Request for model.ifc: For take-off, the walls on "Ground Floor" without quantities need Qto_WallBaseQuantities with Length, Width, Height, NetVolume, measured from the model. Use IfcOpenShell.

First a look at what the model holds.

```python
import ifcopenshell
import ifcopenshell.util.element
import ifcopenshell.util.unit

model = ifcopenshell.open("model.ifc")
print(model.schema)
for unit_type in ("LENGTHUNIT", "AREAUNIT", "VOLUMEUNIT"):
    print(unit_type, ifcopenshell.util.unit.calculate_unit_scale(model, unit_type))
storey = next(s for s in model.by_type("IfcBuildingStorey") if s.Name == "Ground Floor")
walls = [e for e in ifcopenshell.util.element.get_decomposition(storey) if e.is_a("IfcWall")]
for e in sorted(walls, key=lambda e: e.id()):
    print(e.id(), e.is_a(), e.Name, list(ifcopenshell.util.element.get_psets(e, qtos_only=True)), sep=" | ")
```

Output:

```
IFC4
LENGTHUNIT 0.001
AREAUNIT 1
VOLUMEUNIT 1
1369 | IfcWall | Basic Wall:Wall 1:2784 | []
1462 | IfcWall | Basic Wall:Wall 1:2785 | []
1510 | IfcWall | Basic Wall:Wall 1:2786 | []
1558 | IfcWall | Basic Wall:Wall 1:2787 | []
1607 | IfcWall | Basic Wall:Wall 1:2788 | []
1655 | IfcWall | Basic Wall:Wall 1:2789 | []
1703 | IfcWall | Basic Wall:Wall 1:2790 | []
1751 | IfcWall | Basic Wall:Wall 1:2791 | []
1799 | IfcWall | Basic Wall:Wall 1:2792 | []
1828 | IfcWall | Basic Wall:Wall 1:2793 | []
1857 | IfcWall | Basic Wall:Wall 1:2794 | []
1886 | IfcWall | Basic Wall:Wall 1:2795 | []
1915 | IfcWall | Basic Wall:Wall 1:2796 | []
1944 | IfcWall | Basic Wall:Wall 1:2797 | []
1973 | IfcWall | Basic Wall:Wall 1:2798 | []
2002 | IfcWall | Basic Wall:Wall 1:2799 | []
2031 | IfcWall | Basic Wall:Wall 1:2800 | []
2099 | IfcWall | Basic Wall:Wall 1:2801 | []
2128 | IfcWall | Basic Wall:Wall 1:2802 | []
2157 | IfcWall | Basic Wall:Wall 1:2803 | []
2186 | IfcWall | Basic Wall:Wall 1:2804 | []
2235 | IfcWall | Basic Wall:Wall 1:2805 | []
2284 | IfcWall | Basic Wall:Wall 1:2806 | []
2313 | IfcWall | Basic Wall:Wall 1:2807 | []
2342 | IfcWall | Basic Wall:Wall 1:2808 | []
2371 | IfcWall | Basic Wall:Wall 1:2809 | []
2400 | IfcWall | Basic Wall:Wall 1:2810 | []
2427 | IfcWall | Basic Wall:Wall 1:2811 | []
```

```python
import ifcopenshell
import ifcopenshell.api.pset
import ifcopenshell.geom
import ifcopenshell.util.element
import ifcopenshell.util.shape
import ifcopenshell.util.unit

model = ifcopenshell.open("model.ifc")
unit_scale = ifcopenshell.util.unit.calculate_unit_scale(model)
volume_scale = ifcopenshell.util.unit.calculate_unit_scale(model, "VOLUMEUNIT")
settings = ifcopenshell.geom.settings()

storey = next(s for s in model.by_type("IfcBuildingStorey") if s.Name == "Ground Floor")
walls = [e for e in ifcopenshell.util.element.get_decomposition(storey) if e.is_a("IfcWall")]

for e in sorted(walls, key=lambda e: e.id()):
    if ifcopenshell.util.element.get_psets(e, qtos_only=True, should_inherit=False):
        continue
    # Geometry comes back in metres, in the element's own axes.
    shape = ifcopenshell.geom.create_shape(settings, e)
    values = {
        "Length": ifcopenshell.util.shape.get_x(shape.geometry) / unit_scale,
        "Width": ifcopenshell.util.shape.get_y(shape.geometry) / unit_scale,
        "Height": ifcopenshell.util.shape.get_z(shape.geometry) / unit_scale,
        "NetVolume": ifcopenshell.util.shape.get_volume(shape.geometry) / volume_scale,
    }
    qto = ifcopenshell.api.pset.add_qto(model, product=e, name="Qto_WallBaseQuantities")
    ifcopenshell.api.pset.edit_qto(model, qto=qto, properties=values)
    print(e.id(), {k: round(v, 3) for k, v in values.items()})

model.write("model_rev.ifc")
```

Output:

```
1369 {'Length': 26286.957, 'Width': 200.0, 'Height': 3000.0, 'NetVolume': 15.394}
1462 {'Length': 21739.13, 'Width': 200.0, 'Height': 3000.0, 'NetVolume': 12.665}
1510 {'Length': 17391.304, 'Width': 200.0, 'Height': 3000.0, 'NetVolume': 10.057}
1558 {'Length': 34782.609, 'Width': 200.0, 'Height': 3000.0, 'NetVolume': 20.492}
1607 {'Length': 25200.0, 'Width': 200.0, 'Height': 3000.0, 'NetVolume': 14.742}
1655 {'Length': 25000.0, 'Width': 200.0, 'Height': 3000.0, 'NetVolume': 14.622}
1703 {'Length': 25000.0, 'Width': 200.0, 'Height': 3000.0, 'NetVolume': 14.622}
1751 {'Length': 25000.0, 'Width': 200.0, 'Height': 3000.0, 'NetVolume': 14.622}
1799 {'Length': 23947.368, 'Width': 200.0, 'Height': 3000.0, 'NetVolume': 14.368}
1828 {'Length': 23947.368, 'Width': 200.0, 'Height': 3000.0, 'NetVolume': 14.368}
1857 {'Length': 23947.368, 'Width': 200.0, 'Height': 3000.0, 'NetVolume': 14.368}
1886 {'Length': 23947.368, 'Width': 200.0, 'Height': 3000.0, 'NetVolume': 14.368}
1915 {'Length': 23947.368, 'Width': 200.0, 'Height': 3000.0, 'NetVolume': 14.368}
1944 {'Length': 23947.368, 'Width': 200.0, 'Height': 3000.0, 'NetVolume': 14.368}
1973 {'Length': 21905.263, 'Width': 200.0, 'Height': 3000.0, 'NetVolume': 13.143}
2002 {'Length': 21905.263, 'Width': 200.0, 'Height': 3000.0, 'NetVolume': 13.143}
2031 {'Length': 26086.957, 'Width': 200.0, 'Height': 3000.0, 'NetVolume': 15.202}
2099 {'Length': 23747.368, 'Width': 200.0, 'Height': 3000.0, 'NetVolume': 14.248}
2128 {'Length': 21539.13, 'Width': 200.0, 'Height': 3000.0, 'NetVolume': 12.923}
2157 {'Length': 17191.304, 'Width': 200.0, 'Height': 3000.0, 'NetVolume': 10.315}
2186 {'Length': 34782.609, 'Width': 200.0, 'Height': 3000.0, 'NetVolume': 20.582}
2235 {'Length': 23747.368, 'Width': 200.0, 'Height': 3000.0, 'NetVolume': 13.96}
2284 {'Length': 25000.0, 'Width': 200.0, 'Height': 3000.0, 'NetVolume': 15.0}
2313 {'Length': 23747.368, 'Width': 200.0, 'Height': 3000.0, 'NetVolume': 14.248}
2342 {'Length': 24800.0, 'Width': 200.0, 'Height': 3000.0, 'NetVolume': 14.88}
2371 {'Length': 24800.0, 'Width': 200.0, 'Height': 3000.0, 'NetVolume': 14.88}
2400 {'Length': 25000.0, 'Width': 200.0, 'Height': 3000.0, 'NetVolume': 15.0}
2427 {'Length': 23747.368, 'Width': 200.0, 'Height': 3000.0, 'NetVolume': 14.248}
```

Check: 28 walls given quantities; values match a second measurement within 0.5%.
